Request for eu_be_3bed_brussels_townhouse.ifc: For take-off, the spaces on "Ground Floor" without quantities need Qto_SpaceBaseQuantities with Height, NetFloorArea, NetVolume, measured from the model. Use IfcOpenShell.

First a look at what the model holds.

```python
import ifcopenshell
import ifcopenshell.util.element
import ifcopenshell.util.unit

model = ifcopenshell.open("eu_be_3bed_brussels_townhouse.ifc")
print(model.schema)
for unit_type in ("LENGTHUNIT", "AREAUNIT", "VOLUMEUNIT"):
    print(unit_type, ifcopenshell.util.unit.calculate_unit_scale(model, unit_type))
storey = next(s for s in model.by_type("IfcBuildingStorey") if s.Name == "Ground Floor")
spaces = [e for e in ifcopenshell.util.element.get_decomposition(storey) if e.is_a("IfcSpace")]
for e in sorted(spaces, key=lambda e: e.id()):
    print(e.id(), e.is_a(), e.Name, list(ifcopenshell.util.element.get_psets(e, qtos_only=True)), sep=" | ")
```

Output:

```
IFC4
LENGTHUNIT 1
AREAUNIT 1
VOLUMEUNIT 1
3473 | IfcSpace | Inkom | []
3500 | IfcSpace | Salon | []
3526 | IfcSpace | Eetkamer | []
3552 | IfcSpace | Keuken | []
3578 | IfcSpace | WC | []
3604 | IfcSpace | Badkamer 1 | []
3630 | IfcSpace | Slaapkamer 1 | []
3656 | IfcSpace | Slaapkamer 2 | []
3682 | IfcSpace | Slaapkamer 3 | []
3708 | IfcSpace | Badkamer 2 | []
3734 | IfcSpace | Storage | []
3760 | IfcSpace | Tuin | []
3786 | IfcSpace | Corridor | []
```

```python
import ifcopenshell
import ifcopenshell.api.pset
import ifcopenshell.geom
import ifcopenshell.util.element
import ifcopenshell.util.shape
import ifcopenshell.util.unit

model = ifcopenshell.open("eu_be_3bed_brussels_townhouse.ifc")
unit_scale = ifcopenshell.util.unit.calculate_unit_scale(model)
area_scale = ifcopenshell.util.unit.calculate_unit_scale(model, "AREAUNIT")
volume_scale = ifcopenshell.util.unit.calculate_unit_scale(model, "VOLUMEUNIT")
settings = ifcopenshell.geom.settings()

storey = next(s for s in model.by_type("IfcBuildingStorey") if s.Name == "Ground Floor")
spaces = [e for e in ifcopenshell.util.element.get_decomposition(storey) if e.is_a("IfcSpace")]

for e in sorted(spaces, key=lambda e: e.id()):
    if ifcopenshell.util.element.get_psets(e, qtos_only=True, should_inherit=False):
        continue
    # Geometry comes back in metres, in the element's own axes.
    shape = ifcopenshell.geom.create_shape(settings, e)
    values = {
        "Height": ifcopenshell.util.shape.get_z(shape.geometry) / unit_scale,
        "NetFloorArea": ifcopenshell.util.shape.get_footprint_area(shape.geometry) / area_scale,
        "NetVolume": ifcopenshell.util.shape.get_volume(shape.geometry) / volume_scale,
    }
    qto = ifcopenshell.api.pset.add_qto(model, product=e, name="Qto_SpaceBaseQuantities")
    ifcopenshell.api.pset.edit_qto(model, qto=qto, properties=values)
    print(e.id(), {k: round(v, 3) for k, v in values.items()})

model.write("eu_be_3bed_brussels_townhouse_rev.ifc")
```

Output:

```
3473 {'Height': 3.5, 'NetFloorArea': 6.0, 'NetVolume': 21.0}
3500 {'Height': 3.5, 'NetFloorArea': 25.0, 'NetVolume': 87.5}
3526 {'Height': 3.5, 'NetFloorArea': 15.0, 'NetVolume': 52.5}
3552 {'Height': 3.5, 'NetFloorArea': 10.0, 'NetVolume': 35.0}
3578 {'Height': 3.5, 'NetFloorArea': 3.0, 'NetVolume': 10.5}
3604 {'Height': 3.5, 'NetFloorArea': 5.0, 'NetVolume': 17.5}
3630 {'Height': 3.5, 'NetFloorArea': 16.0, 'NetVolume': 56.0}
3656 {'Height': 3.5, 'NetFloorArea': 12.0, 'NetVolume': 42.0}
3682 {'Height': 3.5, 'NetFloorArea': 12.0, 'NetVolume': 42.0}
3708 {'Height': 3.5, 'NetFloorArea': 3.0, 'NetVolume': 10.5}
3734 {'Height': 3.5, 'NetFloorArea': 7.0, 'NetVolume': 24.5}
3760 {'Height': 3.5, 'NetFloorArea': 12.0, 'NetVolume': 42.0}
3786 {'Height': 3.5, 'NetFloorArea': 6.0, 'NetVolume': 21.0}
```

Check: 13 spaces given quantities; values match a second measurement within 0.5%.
